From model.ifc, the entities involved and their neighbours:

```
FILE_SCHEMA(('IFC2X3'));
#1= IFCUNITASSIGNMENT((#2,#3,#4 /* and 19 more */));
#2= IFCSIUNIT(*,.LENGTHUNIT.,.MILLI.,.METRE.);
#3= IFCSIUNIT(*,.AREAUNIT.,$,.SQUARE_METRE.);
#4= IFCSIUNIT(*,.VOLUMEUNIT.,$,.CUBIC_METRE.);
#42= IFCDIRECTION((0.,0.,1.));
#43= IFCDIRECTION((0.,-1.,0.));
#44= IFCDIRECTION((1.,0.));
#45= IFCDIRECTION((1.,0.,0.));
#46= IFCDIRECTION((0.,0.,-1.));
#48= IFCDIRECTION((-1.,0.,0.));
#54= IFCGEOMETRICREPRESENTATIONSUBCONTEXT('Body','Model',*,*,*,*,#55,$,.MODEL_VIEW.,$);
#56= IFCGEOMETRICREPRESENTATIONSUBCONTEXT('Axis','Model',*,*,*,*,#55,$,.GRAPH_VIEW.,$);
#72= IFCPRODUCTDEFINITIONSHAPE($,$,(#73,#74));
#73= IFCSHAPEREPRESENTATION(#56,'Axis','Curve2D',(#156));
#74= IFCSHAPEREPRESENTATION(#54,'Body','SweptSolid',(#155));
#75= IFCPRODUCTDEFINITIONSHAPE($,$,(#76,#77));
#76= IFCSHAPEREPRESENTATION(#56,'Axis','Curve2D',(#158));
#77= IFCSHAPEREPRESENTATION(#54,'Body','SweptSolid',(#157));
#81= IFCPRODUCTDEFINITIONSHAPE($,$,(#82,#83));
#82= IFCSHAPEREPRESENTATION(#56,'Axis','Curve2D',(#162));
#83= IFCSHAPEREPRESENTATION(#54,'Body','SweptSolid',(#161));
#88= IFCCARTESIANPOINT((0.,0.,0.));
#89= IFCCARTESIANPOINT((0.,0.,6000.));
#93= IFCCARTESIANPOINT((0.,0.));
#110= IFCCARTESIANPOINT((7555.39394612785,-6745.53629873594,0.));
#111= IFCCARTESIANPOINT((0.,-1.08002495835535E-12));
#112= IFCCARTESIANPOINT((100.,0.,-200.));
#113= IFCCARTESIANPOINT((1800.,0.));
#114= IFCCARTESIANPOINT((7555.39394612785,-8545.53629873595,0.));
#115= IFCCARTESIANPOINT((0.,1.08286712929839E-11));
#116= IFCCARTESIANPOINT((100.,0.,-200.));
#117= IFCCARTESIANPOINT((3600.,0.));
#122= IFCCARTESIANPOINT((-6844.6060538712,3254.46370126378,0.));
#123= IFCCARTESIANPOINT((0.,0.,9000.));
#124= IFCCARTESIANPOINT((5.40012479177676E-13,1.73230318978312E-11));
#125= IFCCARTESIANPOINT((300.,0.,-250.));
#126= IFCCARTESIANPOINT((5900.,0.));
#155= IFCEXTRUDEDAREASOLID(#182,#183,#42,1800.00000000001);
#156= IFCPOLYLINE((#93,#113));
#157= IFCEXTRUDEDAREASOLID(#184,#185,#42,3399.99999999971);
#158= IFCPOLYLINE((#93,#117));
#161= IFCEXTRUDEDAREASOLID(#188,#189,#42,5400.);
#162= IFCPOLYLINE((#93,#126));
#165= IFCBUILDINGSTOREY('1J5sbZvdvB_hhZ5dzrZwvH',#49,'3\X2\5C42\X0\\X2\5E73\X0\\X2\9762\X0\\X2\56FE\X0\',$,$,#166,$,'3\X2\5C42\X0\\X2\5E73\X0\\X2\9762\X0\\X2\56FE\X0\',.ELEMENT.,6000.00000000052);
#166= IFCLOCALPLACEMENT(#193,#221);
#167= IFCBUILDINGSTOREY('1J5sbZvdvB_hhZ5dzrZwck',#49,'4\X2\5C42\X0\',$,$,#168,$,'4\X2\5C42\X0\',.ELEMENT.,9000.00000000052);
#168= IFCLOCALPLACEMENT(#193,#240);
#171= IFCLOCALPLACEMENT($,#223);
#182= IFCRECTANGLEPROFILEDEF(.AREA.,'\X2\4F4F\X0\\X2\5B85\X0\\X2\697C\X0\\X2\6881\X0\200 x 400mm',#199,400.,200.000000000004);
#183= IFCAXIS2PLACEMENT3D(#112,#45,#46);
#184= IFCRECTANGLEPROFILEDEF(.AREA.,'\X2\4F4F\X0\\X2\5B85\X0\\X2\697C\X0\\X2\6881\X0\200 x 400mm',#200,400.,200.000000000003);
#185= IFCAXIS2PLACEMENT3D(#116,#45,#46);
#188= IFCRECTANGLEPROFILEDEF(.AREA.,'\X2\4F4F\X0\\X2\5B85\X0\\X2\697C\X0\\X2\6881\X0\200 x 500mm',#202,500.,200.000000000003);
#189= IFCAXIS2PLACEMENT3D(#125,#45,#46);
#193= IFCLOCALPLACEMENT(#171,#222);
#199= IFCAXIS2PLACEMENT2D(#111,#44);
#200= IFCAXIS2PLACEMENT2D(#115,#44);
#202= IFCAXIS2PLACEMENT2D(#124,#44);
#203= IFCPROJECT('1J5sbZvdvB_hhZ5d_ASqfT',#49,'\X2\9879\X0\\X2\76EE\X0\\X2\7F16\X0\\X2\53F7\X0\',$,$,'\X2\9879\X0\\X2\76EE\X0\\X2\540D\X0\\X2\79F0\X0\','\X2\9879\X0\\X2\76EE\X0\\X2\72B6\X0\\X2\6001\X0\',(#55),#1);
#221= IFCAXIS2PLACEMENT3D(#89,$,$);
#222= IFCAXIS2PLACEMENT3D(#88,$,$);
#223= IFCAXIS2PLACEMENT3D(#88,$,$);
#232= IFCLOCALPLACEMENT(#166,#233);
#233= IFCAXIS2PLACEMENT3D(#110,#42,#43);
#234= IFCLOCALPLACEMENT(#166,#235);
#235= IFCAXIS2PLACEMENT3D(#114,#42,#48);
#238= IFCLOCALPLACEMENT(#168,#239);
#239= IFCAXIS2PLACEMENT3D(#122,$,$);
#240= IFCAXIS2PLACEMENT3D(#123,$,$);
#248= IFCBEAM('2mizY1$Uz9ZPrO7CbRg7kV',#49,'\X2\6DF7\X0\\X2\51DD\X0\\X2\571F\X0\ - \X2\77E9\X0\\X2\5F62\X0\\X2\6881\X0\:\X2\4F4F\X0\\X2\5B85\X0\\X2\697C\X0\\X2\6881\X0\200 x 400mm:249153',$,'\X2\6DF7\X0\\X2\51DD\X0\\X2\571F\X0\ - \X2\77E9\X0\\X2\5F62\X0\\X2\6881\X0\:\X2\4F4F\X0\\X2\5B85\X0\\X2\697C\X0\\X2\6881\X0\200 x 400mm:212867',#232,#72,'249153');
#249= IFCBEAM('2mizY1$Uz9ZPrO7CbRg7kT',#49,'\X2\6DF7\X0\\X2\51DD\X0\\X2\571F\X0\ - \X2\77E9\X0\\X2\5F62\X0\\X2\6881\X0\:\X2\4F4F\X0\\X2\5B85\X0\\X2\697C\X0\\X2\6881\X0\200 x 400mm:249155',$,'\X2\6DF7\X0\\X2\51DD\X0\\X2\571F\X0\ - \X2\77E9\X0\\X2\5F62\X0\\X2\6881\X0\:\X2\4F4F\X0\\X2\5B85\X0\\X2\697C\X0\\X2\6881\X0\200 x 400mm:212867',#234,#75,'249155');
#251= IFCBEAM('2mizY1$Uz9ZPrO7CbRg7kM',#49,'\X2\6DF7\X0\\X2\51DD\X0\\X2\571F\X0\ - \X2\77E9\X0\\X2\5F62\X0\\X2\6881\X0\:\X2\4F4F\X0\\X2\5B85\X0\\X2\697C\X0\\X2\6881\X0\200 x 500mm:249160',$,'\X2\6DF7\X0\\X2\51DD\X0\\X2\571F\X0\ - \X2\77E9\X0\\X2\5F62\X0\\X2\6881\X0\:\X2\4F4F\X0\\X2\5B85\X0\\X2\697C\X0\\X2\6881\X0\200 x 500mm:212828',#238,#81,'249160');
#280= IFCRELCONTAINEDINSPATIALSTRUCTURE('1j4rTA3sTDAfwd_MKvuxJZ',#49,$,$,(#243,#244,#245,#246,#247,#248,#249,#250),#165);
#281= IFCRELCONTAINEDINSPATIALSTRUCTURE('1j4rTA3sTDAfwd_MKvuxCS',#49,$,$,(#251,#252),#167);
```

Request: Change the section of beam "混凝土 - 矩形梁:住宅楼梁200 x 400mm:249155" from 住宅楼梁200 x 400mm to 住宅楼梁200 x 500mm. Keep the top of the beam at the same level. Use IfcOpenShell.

```python
import ifcopenshell
import ifcopenshell.util.element
import ifcopenshell.util.representation

model = ifcopenshell.open("model.ifc")

member = model.by_guid("2mizY1$Uz9ZPrO7CbRg7kT")
source = next(p for p in model.by_type("IfcRectangleProfileDef") if p.ProfileName == "住宅楼梁200 x 500mm")

body = ifcopenshell.util.representation.get_representation(member, "Model", "Body")
solid = body.Items[0]
old_profile = solid.SweptArea

# Copy the section's sizes but keep this member's own profile position.
profile = ifcopenshell.util.element.copy(model, source)
# Profiles are centred, so shift by half the change in depth to hold the top.
shift = (old_profile.XDim - profile.XDim) / 2
x, y = old_profile.Position.Location.Coordinates
up = (-1.0, 0.0)  # upwards, in the solid's own plane
location = model.createIfcCartesianPoint((x + up[0] * shift, y + up[1] * shift))
profile.Position = model.createIfcAxis2Placement2D(location, old_profile.Position.RefDirection)
solid.SweptArea = profile
if not model.get_total_inverses(old_profile):
    ifcopenshell.util.element.remove_deep2(model, old_profile)
member.Name = member.Name.replace("住宅楼梁200 x 400mm", "住宅楼梁200 x 500mm")
member.ObjectType = member.ObjectType.replace("住宅楼梁200 x 400mm", "住宅楼梁200 x 500mm")

print(solid.SweptArea)

model.write("model-out.ifc")
```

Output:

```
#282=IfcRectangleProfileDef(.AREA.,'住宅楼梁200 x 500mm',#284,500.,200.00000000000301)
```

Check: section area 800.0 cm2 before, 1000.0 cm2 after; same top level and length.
